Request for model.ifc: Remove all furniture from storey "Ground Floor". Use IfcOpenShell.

First a look at what the model holds.

```python
import ifcopenshell
import ifcopenshell.util.element

model = ifcopenshell.open("model.ifc")
print(model.schema)
storey = next(s for s in model.by_type("IfcBuildingStorey") if s.Name == "Ground Floor")
furniture = [e for e in ifcopenshell.util.element.get_decomposition(storey) if e.is_a("IfcFurnishingElement")]
seen = {}
for e in furniture:
    element_type = ifcopenshell.util.element.get_type(e)
    name = element_type.Name if element_type not in (None, e) else None
    seen[name] = seen.get(name, 0) + 1
for name, count in sorted(seen.items(), key=str):
    print(count, "x", name)
```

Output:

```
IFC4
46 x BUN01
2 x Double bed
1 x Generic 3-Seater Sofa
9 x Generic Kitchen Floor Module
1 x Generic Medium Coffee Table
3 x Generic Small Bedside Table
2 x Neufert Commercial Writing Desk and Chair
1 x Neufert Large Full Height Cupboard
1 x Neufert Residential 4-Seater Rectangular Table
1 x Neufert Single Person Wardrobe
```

```python
import ifcopenshell
import ifcopenshell.api.root
import ifcopenshell.util.element

model = ifcopenshell.open("model.ifc")

storey = next(s for s in model.by_type("IfcBuildingStorey") if s.Name == "Ground Floor")
furniture = [e for e in ifcopenshell.util.element.get_decomposition(storey) if e.is_a("IfcFurnishingElement")]

for e in furniture:
    ifcopenshell.api.root.remove_product(model, product=e)
print(len(furniture), "removed")

model.write("model_rev.ifc")
```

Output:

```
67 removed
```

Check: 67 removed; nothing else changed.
